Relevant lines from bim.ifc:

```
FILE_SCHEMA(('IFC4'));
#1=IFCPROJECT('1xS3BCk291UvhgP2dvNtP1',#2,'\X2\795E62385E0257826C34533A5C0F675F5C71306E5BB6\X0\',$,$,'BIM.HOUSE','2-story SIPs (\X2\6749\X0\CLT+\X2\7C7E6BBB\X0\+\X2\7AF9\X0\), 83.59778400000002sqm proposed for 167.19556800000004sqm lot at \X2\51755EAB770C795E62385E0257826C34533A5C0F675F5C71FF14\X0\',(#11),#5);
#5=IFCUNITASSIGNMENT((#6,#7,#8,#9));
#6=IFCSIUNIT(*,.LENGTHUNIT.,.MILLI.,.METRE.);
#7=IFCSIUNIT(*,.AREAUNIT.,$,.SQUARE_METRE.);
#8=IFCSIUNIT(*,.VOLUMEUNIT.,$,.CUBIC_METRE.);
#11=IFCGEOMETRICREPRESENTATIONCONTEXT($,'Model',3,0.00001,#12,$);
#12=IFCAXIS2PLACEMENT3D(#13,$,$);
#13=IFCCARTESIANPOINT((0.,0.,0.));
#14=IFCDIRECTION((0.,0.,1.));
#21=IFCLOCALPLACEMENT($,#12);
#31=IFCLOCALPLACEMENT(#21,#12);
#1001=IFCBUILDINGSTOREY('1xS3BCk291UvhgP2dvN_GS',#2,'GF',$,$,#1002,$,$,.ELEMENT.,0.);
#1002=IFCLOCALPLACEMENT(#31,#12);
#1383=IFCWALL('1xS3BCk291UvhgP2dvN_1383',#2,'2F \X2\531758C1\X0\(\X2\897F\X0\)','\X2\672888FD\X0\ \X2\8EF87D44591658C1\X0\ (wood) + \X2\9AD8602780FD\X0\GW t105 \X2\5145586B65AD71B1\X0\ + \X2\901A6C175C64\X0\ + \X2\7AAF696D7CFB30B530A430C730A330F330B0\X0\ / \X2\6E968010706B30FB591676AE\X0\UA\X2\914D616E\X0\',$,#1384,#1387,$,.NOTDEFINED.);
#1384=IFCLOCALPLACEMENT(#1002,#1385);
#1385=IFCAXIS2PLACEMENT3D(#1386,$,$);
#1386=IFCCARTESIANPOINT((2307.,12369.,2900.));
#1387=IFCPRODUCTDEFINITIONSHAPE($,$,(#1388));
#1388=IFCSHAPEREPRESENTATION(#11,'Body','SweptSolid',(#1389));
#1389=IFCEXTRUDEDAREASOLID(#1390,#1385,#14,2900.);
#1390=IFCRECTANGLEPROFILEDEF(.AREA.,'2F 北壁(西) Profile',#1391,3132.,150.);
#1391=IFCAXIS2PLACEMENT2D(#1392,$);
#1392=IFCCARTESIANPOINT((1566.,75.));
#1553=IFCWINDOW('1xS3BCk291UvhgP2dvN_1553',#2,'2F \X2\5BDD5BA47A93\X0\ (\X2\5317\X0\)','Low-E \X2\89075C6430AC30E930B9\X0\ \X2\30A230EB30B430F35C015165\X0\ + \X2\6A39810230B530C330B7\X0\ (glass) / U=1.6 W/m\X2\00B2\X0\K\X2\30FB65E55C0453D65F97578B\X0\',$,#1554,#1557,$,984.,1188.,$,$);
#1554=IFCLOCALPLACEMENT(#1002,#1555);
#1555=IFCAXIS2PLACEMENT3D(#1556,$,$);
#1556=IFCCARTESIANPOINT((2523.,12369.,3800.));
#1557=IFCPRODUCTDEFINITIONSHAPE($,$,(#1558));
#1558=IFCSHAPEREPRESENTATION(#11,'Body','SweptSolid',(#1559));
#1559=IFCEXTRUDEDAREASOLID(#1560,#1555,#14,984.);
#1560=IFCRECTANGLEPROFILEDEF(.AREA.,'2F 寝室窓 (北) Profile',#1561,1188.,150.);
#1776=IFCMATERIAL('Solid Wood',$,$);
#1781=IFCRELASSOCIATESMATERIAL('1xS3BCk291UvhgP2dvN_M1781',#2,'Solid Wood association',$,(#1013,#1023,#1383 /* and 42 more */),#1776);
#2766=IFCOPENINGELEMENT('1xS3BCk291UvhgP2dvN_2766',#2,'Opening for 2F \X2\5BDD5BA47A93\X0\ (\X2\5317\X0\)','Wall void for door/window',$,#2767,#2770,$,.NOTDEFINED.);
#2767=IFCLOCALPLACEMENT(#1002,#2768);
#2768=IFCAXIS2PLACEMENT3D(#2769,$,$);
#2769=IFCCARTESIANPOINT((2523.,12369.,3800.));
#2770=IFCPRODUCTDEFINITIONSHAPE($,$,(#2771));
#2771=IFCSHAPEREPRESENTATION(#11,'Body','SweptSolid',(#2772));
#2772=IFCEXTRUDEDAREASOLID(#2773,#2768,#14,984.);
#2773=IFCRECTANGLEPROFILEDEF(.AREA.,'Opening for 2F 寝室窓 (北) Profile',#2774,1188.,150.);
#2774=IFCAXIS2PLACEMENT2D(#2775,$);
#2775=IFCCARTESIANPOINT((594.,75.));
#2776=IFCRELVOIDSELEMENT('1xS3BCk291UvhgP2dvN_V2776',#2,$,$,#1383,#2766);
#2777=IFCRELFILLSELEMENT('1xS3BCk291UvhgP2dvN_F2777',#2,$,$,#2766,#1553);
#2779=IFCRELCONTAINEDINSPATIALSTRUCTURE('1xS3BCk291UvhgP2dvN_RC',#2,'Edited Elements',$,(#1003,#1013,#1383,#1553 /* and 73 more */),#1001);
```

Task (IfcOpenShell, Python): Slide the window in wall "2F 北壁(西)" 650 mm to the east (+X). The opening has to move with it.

```python
import ifcopenshell
import ifcopenshell.api.geometry
import ifcopenshell.util.placement
import ifcopenshell.util.unit

model = ifcopenshell.open("bim.ifc")
unit_scale = ifcopenshell.util.unit.calculate_unit_scale(model)

window = model.by_guid("1xS3BCk291UvhgP2dvN_1553")
opening = window.FillsVoids[0].RelatingOpeningElement
wall = opening.VoidsElements[0].RelatingBuildingElement

wall_matrix = ifcopenshell.util.placement.get_local_placement(wall.ObjectPlacement)
shift = wall_matrix[:3, 0] * 0.65 / unit_scale
before = ifcopenshell.util.placement.get_local_placement(window.ObjectPlacement)[:3, 3].copy()

# The window is not placed relative to its opening, so move both.
for product in (opening, window):
    matrix = ifcopenshell.util.placement.get_local_placement(product.ObjectPlacement)
    matrix[:3, 3] += shift
    ifcopenshell.api.geometry.edit_object_placement(model, product=product, matrix=matrix, is_si=False)

after = ifcopenshell.util.placement.get_local_placement(window.ObjectPlacement)[:3, 3]
print("window moved by", (after - before).round(3) + 0.0)

model.write("bim-out.ifc")
```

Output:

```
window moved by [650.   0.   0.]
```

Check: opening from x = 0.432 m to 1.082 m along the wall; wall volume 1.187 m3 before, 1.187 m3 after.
